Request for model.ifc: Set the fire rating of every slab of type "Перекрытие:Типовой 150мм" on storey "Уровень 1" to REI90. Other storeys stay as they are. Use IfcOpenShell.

First a look at what the model holds.

```python
import ifcopenshell
import ifcopenshell.util.element

model = ifcopenshell.open("model.ifc")
print(model.schema)
storey = next(s for s in model.by_type("IfcBuildingStorey") if s.Name == "Уровень 1")
slabs = [e for e in ifcopenshell.util.element.get_decomposition(storey) if e.is_a("IfcSlab")]
seen = {}
for e in slabs:
    element_type = ifcopenshell.util.element.get_type(e)
    key = (element_type.Name if element_type != e and element_type else None, ifcopenshell.util.element.get_pset(e, "Pset_SlabCommon", "FireRating"))
    seen[key] = seen.get(key, 0) + 1
for (name, value), count in sorted(seen.items(), key=str):
    print(count, "x", name, "|", value)
```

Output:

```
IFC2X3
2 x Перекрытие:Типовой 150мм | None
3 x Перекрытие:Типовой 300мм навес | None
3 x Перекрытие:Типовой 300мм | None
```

```python
import ifcopenshell
import ifcopenshell.api.pset
import ifcopenshell.util.element

model = ifcopenshell.open("model.ifc")

storey = next(s for s in model.by_type("IfcBuildingStorey") if s.Name == "Уровень 1")
slabs = [e for e in ifcopenshell.util.element.get_decomposition(storey) if e.is_a("IfcSlab")]

count = 0
for e in slabs:
    element_type = ifcopenshell.util.element.get_type(e)
    if element_type in (None, e) or element_type.Name != "Перекрытие:Типовой 150мм":
        continue
    # add_pset returns the element's existing set when there is one.
    pset = ifcopenshell.api.pset.add_pset(model, product=e, name="Pset_SlabCommon")
    ifcopenshell.api.pset.edit_pset(model, pset=pset, properties={"FireRating": "REI90"})
    count += 1

print(count, "slabs updated")

model.write("model_updated.ifc")
```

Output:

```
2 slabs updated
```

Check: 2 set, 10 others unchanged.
